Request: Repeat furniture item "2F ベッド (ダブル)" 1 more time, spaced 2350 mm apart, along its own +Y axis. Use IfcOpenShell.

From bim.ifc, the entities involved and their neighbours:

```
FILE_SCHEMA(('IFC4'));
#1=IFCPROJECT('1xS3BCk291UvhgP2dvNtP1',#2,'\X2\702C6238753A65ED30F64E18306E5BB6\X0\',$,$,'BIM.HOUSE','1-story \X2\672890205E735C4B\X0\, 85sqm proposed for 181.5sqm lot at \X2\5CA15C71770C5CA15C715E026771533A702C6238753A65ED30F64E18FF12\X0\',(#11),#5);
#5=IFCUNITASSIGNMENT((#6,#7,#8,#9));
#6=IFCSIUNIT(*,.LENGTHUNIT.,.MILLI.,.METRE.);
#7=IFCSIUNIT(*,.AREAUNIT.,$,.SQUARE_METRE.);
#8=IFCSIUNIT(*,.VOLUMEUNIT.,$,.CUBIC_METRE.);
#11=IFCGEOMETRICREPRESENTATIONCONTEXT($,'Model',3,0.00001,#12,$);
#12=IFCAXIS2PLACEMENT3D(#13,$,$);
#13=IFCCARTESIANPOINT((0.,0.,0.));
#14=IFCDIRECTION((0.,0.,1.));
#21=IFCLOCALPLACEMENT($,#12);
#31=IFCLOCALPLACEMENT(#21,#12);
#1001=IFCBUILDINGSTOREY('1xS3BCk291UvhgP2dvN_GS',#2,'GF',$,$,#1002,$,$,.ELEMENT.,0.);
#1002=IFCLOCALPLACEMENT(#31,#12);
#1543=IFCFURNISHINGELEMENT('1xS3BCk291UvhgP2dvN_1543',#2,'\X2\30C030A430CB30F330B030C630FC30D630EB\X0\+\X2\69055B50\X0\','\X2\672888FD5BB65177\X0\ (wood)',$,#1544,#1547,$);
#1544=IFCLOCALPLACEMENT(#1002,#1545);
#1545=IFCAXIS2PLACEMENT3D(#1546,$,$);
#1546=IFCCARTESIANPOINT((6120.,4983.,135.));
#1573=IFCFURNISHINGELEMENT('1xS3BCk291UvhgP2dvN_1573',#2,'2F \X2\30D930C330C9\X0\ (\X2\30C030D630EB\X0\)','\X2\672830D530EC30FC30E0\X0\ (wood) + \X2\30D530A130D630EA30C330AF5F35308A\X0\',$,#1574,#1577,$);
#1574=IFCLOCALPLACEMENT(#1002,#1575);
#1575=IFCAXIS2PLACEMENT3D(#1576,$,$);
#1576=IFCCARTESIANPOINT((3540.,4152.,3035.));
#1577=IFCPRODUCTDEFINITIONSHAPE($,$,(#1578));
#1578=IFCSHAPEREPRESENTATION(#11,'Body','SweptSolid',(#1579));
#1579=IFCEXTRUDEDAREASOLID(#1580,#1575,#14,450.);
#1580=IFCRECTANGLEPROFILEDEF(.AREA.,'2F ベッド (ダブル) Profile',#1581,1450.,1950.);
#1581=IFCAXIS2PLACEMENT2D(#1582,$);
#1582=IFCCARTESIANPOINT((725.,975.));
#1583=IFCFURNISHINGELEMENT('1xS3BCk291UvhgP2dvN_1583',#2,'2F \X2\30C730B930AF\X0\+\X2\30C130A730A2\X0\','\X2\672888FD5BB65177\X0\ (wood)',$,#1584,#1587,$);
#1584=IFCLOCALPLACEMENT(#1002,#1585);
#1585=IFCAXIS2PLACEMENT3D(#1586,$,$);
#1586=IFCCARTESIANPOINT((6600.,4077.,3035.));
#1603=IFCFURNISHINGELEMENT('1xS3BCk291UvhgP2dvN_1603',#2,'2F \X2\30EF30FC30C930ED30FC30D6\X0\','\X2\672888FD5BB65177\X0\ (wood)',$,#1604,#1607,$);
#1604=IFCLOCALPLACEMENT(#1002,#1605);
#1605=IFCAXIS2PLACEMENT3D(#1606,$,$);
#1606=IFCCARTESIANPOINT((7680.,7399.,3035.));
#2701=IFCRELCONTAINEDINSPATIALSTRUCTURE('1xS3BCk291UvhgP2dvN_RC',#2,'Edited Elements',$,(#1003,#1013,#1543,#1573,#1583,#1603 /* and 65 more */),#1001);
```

```python
import ifcopenshell
import ifcopenshell.api.geometry
import ifcopenshell.api.root
import ifcopenshell.util.element
import ifcopenshell.util.placement

model = ifcopenshell.open("bim.ifc")


def reuse_history(source, copy):
    """copy_class also copies each property set's owner history, people and application; keep the originals."""
    for rel in copy.IsDefinedBy:
        if rel.is_a("IfcRelDefinesByProperties") and (history := rel.RelatingPropertyDefinition.OwnerHistory):
            rel.RelatingPropertyDefinition.OwnerHistory = source.OwnerHistory
            ifcopenshell.util.element.remove_deep2(model, history)


source = model.by_guid("1xS3BCk291UvhgP2dvN_1573")
base = ifcopenshell.util.placement.get_local_placement(source.ObjectPlacement)
step = base[:3, 1] * 2350.0

for i in range(1, 2):
    copy = ifcopenshell.api.root.copy_class(model, product=source)
    copy.Representation = ifcopenshell.util.element.copy_deep(
        model, source.Representation, exclude=["IfcGeometricRepresentationContext", "IfcRepresentationMap"]
    )
    reuse_history(source, copy)
    matrix = base.copy()
    matrix[:3, 3] += i * step
    print("added at", matrix[:3, 3].round(3) + 0.0)
    ifcopenshell.api.geometry.edit_object_placement(model, product=copy, matrix=matrix, is_si=False)

model.write("bim-out.ifc")
```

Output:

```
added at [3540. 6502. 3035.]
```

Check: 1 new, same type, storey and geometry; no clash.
